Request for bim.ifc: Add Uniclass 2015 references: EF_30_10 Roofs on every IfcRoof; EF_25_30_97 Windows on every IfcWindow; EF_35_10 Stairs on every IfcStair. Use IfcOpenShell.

First a look at what the model holds.

```python
import ifcopenshell

model = ifcopenshell.open("bim.ifc")
print(model.schema)
print("classifications:", [c.Name for c in model.by_type("IfcClassification")])
for ifc_class in ("IfcDoor", "IfcRoof", "IfcStair", "IfcWall", "IfcWindow"):
    print(ifc_class, len(model.by_type(ifc_class)))
```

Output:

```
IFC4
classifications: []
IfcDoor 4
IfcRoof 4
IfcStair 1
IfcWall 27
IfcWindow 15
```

```python
import ifcopenshell
import ifcopenshell.api.classification

model = ifcopenshell.open("bim.ifc")

system = ifcopenshell.api.classification.add_classification(model, classification="Uniclass 2015")

codes = {
    "IfcRoof": ("EF_30_10", "Roofs"),
    "IfcWindow": ("EF_25_30_97", "Windows"),
    "IfcStair": ("EF_35_10", "Stairs"),
}
for ifc_class, (code, name) in codes.items():
    products = model.by_type(ifc_class)
    ifcopenshell.api.classification.add_reference(
        model, products=products, classification=system, identification=code, name=name
    )
    print(code, len(products))

model.write("bim_rev.ifc")
```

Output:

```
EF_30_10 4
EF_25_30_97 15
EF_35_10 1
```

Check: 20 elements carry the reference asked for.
